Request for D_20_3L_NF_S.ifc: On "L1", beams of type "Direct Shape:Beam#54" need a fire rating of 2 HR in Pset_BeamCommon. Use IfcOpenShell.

First a look at what the model holds.

```python
import ifcopenshell
import ifcopenshell.util.element

model = ifcopenshell.open("D_20_3L_NF_S.ifc")
print(model.schema)
storey = next(s for s in model.by_type("IfcBuildingStorey") if s.Name == "L1")
beams = [e for e in ifcopenshell.util.element.get_decomposition(storey) if e.is_a("IfcBeam")]
seen = {}
for e in beams:
    element_type = ifcopenshell.util.element.get_type(e)
    key = (element_type.Name if element_type != e and element_type else None, ifcopenshell.util.element.get_pset(e, "Pset_BeamCommon", "FireRating"))
    seen[key] = seen.get(key, 0) + 1
for (name, value), count in sorted(seen.items(), key=str):
    print(count, "x", name, "|", value)
```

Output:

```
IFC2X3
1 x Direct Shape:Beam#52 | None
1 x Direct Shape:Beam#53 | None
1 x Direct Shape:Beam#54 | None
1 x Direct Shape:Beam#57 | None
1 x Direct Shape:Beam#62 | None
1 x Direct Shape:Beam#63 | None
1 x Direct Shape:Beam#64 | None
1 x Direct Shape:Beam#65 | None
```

```python
import ifcopenshell
import ifcopenshell.api.pset
import ifcopenshell.util.element

model = ifcopenshell.open("D_20_3L_NF_S.ifc")

storey = next(s for s in model.by_type("IfcBuildingStorey") if s.Name == "L1")
beams = [e for e in ifcopenshell.util.element.get_decomposition(storey) if e.is_a("IfcBeam")]

count = 0
for e in beams:
    element_type = ifcopenshell.util.element.get_type(e)
    if element_type in (None, e) or element_type.Name != "Direct Shape:Beam#54":
        continue
    # add_pset returns the element's existing set when there is one.
    pset = ifcopenshell.api.pset.add_pset(model, product=e, name="Pset_BeamCommon")
    ifcopenshell.api.pset.edit_pset(model, pset=pset, properties={"FireRating": "2 HR"})
    count += 1

print(count, "beams updated")

model.write("D_20_3L_NF_S-out.ifc")
```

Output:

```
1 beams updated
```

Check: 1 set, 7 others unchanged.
